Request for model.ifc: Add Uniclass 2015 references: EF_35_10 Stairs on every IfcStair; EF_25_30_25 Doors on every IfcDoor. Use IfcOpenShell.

First a look at what the model holds.

```python
import ifcopenshell

model = ifcopenshell.open("model.ifc")
print(model.schema)
print("classifications:", [c.Name for c in model.by_type("IfcClassification")])
for ifc_class in ("IfcDoor", "IfcRoof", "IfcStair", "IfcWall", "IfcWindow"):
    print(ifc_class, len(model.by_type(ifc_class)))
```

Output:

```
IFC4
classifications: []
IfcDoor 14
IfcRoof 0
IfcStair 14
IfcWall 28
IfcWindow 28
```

```python
import ifcopenshell
import ifcopenshell.api.classification

model = ifcopenshell.open("model.ifc")

system = ifcopenshell.api.classification.add_classification(model, classification="Uniclass 2015")

codes = {
    "IfcStair": ("EF_35_10", "Stairs"),
    "IfcDoor": ("EF_25_30_25", "Doors"),
}
for ifc_class, (code, name) in codes.items():
    products = model.by_type(ifc_class)
    ifcopenshell.api.classification.add_reference(
        model, products=products, classification=system, identification=code, name=name
    )
    print(code, len(products))

model.write("model_edited.ifc")
```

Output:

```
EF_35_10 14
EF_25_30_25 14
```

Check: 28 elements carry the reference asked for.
